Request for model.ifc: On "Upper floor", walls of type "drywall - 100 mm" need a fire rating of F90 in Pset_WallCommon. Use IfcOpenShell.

First a look at what the model holds.

```python
import ifcopenshell
import ifcopenshell.util.element

model = ifcopenshell.open("model.ifc")
print(model.schema)
storey = next(s for s in model.by_type("IfcBuildingStorey") if s.Name == "Upper floor")
walls = [e for e in ifcopenshell.util.element.get_decomposition(storey) if e.is_a("IfcWall")]
seen = {}
for e in walls:
    element_type = ifcopenshell.util.element.get_type(e)
    key = (element_type.Name if element_type != e and element_type else None, ifcopenshell.util.element.get_pset(e, "Pset_WallCommon", "FireRating"))
    seen[key] = seen.get(key, 0) + 1
for (name, value), count in sorted(seen.items(), key=str):
    print(count, "x", name, "|", value)
```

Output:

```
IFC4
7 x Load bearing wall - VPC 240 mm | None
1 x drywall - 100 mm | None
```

```python
import ifcopenshell
import ifcopenshell.api.pset
import ifcopenshell.util.element

model = ifcopenshell.open("model.ifc")

storey = next(s for s in model.by_type("IfcBuildingStorey") if s.Name == "Upper floor")
walls = [e for e in ifcopenshell.util.element.get_decomposition(storey) if e.is_a("IfcWall")]

count = 0
for e in walls:
    element_type = ifcopenshell.util.element.get_type(e)
    if element_type in (None, e) or element_type.Name != "drywall - 100 mm":
        continue
    # add_pset returns the element's existing set when there is one.
    pset = ifcopenshell.api.pset.add_pset(model, product=e, name="Pset_WallCommon")
    ifcopenshell.api.pset.edit_pset(model, pset=pset, properties={"FireRating": "F90"})
    count += 1

print(count, "walls updated")

model.write("model_v2.ifc")
```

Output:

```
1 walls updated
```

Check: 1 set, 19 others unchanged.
